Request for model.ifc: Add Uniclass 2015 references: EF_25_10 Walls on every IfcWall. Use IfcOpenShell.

First a look at what the model holds.

```python
import ifcopenshell

model = ifcopenshell.open("model.ifc")
print(model.schema)
print("classifications:", [c.Name for c in model.by_type("IfcClassification")])
for ifc_class in ("IfcDoor", "IfcRoof", "IfcStair", "IfcWall", "IfcWindow"):
    print(ifc_class, len(model.by_type(ifc_class)))
```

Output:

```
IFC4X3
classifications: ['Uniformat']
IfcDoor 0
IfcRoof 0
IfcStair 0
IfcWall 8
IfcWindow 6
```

```python
import ifcopenshell
import ifcopenshell.api.classification

model = ifcopenshell.open("model.ifc")

system = ifcopenshell.api.classification.add_classification(model, classification="Uniclass 2015")

codes = {
    "IfcWall": ("EF_25_10", "Walls"),
}
for ifc_class, (code, name) in codes.items():
    products = model.by_type(ifc_class)
    ifcopenshell.api.classification.add_reference(
        model, products=products, classification=system, identification=code, name=name
    )
    print(code, len(products))

model.write("model_updated.ifc")
```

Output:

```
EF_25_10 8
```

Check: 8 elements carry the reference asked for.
